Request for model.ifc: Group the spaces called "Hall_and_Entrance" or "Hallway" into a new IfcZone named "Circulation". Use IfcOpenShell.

First a look at what the model holds.

```python
import ifcopenshell

model = ifcopenshell.open("model.ifc")
print(model.schema)
seen = {}
for space in model.by_type("IfcSpace"):
    seen[space.Name] = seen.get(space.Name, 0) + 1
for name, count in sorted(seen.items(), key=str):
    print(count, "x", name)
print("zones:", [z.Name for z in model.by_type("IfcZone")][:20])
```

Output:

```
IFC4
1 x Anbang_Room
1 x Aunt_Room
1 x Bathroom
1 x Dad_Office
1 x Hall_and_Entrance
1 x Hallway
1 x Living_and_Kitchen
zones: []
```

```python
import ifcopenshell
import ifcopenshell.api.group
import ifcopenshell.api.root

model = ifcopenshell.open("model.ifc")

names = {"Hall_and_Entrance", "Hallway"}
spaces = [s for s in model.by_type("IfcSpace") if s.Name in names]

zone = ifcopenshell.api.root.create_entity(model, ifc_class="IfcZone", name="Circulation")
ifcopenshell.api.group.assign_group(model, products=spaces, group=zone)
print(len(spaces), "spaces in", zone.Name)

model.write("model-out.ifc")
```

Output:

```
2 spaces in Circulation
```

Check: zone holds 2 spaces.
